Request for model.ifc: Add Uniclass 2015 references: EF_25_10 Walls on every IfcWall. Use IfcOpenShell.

First a look at what the model holds.

```python
import ifcopenshell

model = ifcopenshell.open("model.ifc")
print(model.schema)
print("classifications:", [c.Name for c in model.by_type("IfcClassification")])
for ifc_class in ("IfcDoor", "IfcRoof", "IfcStair", "IfcWall", "IfcWindow"):
    print(ifc_class, len(model.by_type(ifc_class)))
```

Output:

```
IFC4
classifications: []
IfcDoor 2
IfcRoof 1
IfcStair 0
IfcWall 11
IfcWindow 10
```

```python
import ifcopenshell
import ifcopenshell.api.classification

model = ifcopenshell.open("model.ifc")

system = ifcopenshell.api.classification.add_classification(model, classification="Uniclass 2015")

codes = {
    "IfcWall": ("EF_25_10", "Walls"),
}
for ifc_class, (code, name) in codes.items():
    products = model.by_type(ifc_class)
    ifcopenshell.api.classification.add_reference(
        model, products=products, classification=system, identification=code, name=name
    )
    print(code, len(products))

model.write("model-out.ifc")
```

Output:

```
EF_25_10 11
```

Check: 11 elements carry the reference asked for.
